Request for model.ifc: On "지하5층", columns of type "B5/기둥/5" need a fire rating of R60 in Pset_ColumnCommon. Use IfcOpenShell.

First a look at what the model holds.

```python
import ifcopenshell
import ifcopenshell.util.element

model = ifcopenshell.open("model.ifc")
print(model.schema)
storey = next(s for s in model.by_type("IfcBuildingStorey") if s.Name == "지하5층")
columns = [e for e in ifcopenshell.util.element.get_decomposition(storey) if e.is_a("IfcColumn")]
seen = {}
for e in columns:
    element_type = ifcopenshell.util.element.get_type(e)
    key = (element_type.Name if element_type != e and element_type else None, ifcopenshell.util.element.get_pset(e, "Pset_ColumnCommon", "FireRating"))
    seen[key] = seen.get(key, 0) + 1
for (name, value), count in sorted(seen.items(), key=str):
    print(count, "x", name, "|", value)
```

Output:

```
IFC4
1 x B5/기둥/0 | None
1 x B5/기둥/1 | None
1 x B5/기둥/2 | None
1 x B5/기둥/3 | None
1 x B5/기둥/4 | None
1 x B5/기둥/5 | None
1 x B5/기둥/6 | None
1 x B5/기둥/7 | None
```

```python
import ifcopenshell
import ifcopenshell.api.pset
import ifcopenshell.util.element

model = ifcopenshell.open("model.ifc")

storey = next(s for s in model.by_type("IfcBuildingStorey") if s.Name == "지하5층")
columns = [e for e in ifcopenshell.util.element.get_decomposition(storey) if e.is_a("IfcColumn")]

count = 0
for e in columns:
    element_type = ifcopenshell.util.element.get_type(e)
    if element_type in (None, e) or element_type.Name != "B5/기둥/5":
        continue
    # add_pset returns the element's existing set when there is one.
    pset = ifcopenshell.api.pset.add_pset(model, product=e, name="Pset_ColumnCommon")
    ifcopenshell.api.pset.edit_pset(model, pset=pset, properties={"FireRating": "R60"})
    count += 1

print(count, "columns updated")

model.write("model_edited.ifc")
```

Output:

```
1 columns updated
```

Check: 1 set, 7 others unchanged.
